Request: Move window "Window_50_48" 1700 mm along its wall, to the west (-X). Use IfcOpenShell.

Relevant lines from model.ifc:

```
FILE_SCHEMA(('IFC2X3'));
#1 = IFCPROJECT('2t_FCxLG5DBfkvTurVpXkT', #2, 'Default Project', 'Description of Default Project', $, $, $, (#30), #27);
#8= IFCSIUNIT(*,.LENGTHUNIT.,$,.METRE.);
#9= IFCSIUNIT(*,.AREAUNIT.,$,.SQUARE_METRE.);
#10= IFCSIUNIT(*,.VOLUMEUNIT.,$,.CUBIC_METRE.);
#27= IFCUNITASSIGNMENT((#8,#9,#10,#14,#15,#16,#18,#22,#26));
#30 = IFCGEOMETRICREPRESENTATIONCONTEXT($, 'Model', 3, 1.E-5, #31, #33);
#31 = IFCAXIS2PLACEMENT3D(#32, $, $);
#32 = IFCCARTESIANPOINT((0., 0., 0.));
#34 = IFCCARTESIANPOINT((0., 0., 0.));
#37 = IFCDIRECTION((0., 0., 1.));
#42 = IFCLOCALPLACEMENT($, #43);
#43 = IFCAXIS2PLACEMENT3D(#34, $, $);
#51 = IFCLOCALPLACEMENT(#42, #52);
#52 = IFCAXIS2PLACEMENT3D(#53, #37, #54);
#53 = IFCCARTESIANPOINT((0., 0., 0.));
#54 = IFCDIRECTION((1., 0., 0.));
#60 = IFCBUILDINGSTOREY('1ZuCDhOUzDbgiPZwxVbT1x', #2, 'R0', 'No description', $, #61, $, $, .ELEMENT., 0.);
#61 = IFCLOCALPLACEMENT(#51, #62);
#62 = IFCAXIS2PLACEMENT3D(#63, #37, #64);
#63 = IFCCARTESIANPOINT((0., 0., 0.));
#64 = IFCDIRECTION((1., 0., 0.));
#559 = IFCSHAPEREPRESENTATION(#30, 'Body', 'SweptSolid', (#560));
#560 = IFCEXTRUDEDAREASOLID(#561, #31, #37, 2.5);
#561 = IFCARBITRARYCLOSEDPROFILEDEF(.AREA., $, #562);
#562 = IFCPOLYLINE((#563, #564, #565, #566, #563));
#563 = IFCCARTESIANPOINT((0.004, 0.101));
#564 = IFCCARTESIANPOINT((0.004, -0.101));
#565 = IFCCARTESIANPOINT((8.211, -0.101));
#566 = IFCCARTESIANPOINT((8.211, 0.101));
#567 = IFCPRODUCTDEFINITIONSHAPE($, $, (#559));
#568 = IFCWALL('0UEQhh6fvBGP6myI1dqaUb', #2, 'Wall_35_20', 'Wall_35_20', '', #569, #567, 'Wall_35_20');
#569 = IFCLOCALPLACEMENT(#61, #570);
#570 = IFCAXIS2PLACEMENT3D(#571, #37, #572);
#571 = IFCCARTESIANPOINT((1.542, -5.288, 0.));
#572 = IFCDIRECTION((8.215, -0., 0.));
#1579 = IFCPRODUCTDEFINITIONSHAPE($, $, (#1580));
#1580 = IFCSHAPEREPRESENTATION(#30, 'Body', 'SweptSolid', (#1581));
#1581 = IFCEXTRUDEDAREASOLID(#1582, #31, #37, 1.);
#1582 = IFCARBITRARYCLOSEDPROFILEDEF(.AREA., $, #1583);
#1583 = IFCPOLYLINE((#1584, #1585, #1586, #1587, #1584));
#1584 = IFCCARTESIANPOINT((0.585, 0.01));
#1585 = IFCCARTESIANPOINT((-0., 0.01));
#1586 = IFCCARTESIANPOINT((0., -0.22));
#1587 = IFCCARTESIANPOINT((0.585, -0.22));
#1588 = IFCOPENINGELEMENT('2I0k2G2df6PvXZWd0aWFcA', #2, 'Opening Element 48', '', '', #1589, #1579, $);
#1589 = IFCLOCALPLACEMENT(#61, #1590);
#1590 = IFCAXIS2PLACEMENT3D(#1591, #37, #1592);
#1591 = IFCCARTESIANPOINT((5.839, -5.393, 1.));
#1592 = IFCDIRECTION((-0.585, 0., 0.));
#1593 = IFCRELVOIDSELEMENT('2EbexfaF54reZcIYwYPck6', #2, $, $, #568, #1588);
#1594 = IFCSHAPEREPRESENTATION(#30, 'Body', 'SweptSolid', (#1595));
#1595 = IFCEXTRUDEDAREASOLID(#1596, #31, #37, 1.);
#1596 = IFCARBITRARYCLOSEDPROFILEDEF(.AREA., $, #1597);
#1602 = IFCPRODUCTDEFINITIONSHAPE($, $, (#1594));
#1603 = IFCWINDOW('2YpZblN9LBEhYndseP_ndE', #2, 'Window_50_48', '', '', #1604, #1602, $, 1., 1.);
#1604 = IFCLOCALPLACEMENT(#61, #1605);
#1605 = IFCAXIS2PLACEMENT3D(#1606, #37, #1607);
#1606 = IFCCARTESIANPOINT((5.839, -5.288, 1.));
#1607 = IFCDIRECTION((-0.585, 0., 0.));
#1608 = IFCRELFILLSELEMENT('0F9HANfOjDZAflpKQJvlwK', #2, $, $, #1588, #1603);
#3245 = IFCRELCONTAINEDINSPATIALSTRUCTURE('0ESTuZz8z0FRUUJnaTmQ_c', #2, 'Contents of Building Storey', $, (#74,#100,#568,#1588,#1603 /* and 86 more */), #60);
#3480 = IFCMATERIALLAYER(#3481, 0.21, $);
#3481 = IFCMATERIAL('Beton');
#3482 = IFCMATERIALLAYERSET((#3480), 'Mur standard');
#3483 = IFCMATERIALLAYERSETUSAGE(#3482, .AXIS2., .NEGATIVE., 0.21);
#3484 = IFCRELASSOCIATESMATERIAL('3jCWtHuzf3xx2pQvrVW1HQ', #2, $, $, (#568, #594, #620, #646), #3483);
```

```python
import ifcopenshell
import ifcopenshell.api.geometry
import ifcopenshell.util.placement

model = ifcopenshell.open("model.ifc")

window = model.by_guid("2YpZblN9LBEhYndseP_ndE")
opening = window.FillsVoids[0].RelatingOpeningElement
wall = opening.VoidsElements[0].RelatingBuildingElement

wall_matrix = ifcopenshell.util.placement.get_local_placement(wall.ObjectPlacement)
shift = wall_matrix[:3, 0] * -1.7
before = ifcopenshell.util.placement.get_local_placement(window.ObjectPlacement)[:3, 3].copy()

# The window is not placed relative to its opening, so move both.
for product in (opening, window):
    matrix = ifcopenshell.util.placement.get_local_placement(product.ObjectPlacement)
    matrix[:3, 3] += shift
    ifcopenshell.api.geometry.edit_object_placement(model, product=product, matrix=matrix, is_si=False)

after = ifcopenshell.util.placement.get_local_placement(window.ObjectPlacement)[:3, 3]
print("window moved by", (after - before).round(3) + 0.0)

model.write("model_v2.ifc")
```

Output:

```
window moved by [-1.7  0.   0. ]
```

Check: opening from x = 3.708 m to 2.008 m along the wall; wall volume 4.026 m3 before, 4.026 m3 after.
